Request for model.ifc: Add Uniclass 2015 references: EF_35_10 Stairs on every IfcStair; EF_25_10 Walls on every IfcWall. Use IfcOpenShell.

First a look at what the model holds.

```python
import ifcopenshell

model = ifcopenshell.open("model.ifc")
print(model.schema)
print("classifications:", [c.Name for c in model.by_type("IfcClassification")])
for ifc_class in ("IfcDoor", "IfcRoof", "IfcStair", "IfcWall", "IfcWindow"):
    print(ifc_class, len(model.by_type(ifc_class)))
```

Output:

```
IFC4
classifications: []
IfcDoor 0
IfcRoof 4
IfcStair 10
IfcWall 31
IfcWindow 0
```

```python
import ifcopenshell
import ifcopenshell.api.classification

model = ifcopenshell.open("model.ifc")

system = ifcopenshell.api.classification.add_classification(model, classification="Uniclass 2015")

codes = {
    "IfcStair": ("EF_35_10", "Stairs"),
    "IfcWall": ("EF_25_10", "Walls"),
}
for ifc_class, (code, name) in codes.items():
    products = model.by_type(ifc_class)
    ifcopenshell.api.classification.add_reference(
        model, products=products, classification=system, identification=code, name=name
    )
    print(code, len(products))

model.write("model_rev.ifc")
```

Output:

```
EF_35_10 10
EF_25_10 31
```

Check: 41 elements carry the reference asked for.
